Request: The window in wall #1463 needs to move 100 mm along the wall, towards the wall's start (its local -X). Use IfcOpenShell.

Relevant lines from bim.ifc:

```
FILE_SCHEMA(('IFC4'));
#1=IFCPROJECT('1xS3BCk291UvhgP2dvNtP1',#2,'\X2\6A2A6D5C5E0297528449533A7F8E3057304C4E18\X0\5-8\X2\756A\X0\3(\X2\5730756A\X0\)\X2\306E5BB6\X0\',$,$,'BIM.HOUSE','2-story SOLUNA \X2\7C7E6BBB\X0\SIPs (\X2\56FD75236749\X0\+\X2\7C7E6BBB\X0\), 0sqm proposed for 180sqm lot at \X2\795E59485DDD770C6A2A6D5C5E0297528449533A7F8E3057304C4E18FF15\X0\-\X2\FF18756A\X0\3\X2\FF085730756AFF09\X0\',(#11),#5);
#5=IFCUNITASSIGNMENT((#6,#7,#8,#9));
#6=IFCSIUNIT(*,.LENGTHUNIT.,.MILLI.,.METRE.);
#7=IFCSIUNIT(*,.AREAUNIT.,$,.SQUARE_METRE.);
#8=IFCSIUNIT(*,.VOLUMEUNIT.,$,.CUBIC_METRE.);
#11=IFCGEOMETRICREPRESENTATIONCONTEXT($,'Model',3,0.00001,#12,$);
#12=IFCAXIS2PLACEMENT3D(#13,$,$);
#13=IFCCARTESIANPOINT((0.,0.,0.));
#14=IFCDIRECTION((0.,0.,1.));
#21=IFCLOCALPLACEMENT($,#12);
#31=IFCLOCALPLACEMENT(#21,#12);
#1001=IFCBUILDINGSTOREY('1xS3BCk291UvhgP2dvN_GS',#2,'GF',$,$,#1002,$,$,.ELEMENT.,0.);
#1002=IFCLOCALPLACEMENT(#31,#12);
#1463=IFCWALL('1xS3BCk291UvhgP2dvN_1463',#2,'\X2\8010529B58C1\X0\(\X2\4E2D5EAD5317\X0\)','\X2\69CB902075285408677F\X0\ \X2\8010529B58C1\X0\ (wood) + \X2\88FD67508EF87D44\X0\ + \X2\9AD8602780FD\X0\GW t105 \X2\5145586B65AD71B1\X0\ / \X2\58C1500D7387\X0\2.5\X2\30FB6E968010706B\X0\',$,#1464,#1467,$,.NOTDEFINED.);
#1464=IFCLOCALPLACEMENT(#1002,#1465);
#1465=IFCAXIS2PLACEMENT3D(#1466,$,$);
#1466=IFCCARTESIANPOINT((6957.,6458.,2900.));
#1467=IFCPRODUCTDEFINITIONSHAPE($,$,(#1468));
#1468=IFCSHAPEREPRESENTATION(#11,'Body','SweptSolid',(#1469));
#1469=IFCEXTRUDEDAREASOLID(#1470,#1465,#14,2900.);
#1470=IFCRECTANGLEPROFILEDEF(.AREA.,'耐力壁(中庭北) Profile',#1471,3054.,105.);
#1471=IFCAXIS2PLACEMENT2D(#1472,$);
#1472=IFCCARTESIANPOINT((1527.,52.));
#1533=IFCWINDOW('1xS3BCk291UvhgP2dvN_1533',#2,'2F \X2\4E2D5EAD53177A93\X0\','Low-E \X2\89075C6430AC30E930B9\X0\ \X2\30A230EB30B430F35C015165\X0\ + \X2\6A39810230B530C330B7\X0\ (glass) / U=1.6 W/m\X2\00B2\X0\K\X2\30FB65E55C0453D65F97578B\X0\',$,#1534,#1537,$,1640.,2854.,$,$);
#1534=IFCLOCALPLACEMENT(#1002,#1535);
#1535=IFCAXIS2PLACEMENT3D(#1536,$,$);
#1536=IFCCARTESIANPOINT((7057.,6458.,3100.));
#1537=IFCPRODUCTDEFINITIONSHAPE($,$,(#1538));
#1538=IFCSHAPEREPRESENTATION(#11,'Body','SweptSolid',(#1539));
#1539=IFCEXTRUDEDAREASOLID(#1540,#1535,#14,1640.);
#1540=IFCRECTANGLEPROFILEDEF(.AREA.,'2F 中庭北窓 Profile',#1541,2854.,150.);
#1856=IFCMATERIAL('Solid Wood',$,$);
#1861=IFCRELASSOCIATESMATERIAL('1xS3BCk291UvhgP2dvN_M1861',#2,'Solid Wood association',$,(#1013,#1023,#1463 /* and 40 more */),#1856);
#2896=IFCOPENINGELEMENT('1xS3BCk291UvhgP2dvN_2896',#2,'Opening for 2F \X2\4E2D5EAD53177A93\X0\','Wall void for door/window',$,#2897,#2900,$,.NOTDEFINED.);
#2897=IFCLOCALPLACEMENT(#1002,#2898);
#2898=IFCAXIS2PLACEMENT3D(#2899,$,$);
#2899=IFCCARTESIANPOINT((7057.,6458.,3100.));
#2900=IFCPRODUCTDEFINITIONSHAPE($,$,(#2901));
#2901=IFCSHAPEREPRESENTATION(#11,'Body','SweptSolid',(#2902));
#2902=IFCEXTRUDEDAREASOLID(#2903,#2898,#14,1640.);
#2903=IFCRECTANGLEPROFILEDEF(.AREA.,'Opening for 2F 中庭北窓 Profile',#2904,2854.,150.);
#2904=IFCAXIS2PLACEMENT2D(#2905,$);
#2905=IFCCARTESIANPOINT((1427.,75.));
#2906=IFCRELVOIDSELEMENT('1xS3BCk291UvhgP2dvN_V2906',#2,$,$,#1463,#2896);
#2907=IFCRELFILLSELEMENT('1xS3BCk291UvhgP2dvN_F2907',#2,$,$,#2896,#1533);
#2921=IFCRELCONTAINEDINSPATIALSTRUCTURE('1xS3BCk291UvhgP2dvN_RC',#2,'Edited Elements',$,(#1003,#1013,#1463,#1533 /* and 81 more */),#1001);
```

```python
import ifcopenshell
import ifcopenshell.api.geometry
import ifcopenshell.util.placement
import ifcopenshell.util.unit

model = ifcopenshell.open("bim.ifc")
unit_scale = ifcopenshell.util.unit.calculate_unit_scale(model)

window = model.by_id(1533)
opening = window.FillsVoids[0].RelatingOpeningElement
wall = opening.VoidsElements[0].RelatingBuildingElement

wall_matrix = ifcopenshell.util.placement.get_local_placement(wall.ObjectPlacement)
shift = wall_matrix[:3, 0] * -0.1 / unit_scale
before = ifcopenshell.util.placement.get_local_placement(window.ObjectPlacement)[:3, 3].copy()

# The window is not placed relative to its opening, so move both.
for product in (opening, window):
    matrix = ifcopenshell.util.placement.get_local_placement(product.ObjectPlacement)
    matrix[:3, 3] += shift
    ifcopenshell.api.geometry.edit_object_placement(model, product=product, matrix=matrix, is_si=False)

after = ifcopenshell.util.placement.get_local_placement(window.ObjectPlacement)[:3, 3]
print("window moved by", (after - before).round(3) + 0.0)

model.write("bim_updated.ifc")
```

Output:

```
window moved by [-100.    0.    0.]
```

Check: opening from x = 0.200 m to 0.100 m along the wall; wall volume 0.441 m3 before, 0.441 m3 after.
